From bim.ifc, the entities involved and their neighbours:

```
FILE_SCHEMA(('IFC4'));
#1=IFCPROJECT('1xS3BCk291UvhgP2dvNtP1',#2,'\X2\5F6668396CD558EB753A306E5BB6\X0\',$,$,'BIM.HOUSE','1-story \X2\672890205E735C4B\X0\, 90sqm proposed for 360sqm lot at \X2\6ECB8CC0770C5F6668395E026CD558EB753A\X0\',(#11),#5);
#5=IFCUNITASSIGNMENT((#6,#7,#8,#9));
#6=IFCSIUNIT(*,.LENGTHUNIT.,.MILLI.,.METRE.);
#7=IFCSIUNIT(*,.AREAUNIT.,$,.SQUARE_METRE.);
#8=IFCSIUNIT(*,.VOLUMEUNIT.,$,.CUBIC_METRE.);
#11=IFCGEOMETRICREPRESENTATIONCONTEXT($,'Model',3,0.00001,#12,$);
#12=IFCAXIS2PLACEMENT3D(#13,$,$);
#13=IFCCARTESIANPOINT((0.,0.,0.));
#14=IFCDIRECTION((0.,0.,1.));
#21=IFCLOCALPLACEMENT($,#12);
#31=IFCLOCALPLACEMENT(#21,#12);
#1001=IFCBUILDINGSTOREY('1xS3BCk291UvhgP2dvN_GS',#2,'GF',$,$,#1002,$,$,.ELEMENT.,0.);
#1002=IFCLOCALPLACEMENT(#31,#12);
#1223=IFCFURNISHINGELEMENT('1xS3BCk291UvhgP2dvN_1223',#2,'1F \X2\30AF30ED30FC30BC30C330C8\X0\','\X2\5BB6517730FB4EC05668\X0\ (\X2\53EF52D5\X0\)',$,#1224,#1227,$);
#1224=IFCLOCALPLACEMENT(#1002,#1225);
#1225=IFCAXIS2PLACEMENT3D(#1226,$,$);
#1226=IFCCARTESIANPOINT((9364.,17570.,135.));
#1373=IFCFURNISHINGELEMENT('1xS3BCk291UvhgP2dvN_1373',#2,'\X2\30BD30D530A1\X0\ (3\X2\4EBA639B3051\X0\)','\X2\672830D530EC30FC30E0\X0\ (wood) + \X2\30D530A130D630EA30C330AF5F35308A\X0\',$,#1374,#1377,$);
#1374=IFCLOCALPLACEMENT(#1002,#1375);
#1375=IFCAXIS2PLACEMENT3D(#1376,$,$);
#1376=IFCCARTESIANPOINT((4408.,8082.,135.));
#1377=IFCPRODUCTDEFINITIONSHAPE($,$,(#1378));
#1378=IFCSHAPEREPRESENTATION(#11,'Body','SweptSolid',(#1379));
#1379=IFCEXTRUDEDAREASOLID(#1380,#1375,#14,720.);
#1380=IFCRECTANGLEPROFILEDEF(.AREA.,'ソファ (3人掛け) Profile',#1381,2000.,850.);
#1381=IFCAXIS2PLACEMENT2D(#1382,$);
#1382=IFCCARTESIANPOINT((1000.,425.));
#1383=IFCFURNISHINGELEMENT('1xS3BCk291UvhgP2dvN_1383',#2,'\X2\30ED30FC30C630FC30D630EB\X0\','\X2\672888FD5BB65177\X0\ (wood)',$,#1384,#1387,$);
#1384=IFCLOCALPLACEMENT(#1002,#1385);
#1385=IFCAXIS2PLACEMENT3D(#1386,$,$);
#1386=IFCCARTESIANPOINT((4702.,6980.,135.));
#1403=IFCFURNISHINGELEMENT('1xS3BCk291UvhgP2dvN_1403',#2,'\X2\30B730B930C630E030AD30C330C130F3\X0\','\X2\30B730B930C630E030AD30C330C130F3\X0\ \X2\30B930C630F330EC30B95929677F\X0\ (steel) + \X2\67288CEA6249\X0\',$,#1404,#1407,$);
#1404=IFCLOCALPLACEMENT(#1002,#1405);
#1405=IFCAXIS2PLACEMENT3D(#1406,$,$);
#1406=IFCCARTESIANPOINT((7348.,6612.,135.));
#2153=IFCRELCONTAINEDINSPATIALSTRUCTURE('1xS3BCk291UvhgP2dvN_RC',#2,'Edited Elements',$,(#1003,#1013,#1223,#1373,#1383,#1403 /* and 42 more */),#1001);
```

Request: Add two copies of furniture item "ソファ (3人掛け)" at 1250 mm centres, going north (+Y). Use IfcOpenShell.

```python
import numpy as np
import ifcopenshell
import ifcopenshell.api.geometry
import ifcopenshell.api.root
import ifcopenshell.util.element
import ifcopenshell.util.placement

model = ifcopenshell.open("bim.ifc")


def reuse_history(source, copy):
    """copy_class also copies each property set's owner history, people and application; keep the originals."""
    for rel in copy.IsDefinedBy:
        if rel.is_a("IfcRelDefinesByProperties") and (history := rel.RelatingPropertyDefinition.OwnerHistory):
            rel.RelatingPropertyDefinition.OwnerHistory = source.OwnerHistory
            ifcopenshell.util.element.remove_deep2(model, history)


source = model.by_guid("1xS3BCk291UvhgP2dvN_1373")
base = ifcopenshell.util.placement.get_local_placement(source.ObjectPlacement)
step = np.array([0.0, 1.0, 0.0]) * 1250.0

for i in range(1, 3):
    copy = ifcopenshell.api.root.copy_class(model, product=source)
    copy.Representation = ifcopenshell.util.element.copy_deep(
        model, source.Representation, exclude=["IfcGeometricRepresentationContext", "IfcRepresentationMap"]
    )
    reuse_history(source, copy)
    matrix = base.copy()
    matrix[:3, 3] += i * step
    print("added at", matrix[:3, 3].round(3) + 0.0)
    ifcopenshell.api.geometry.edit_object_placement(model, product=copy, matrix=matrix, is_si=False)

model.write("bim_edited.ifc")
```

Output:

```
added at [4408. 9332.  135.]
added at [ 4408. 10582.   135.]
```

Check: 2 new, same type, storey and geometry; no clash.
